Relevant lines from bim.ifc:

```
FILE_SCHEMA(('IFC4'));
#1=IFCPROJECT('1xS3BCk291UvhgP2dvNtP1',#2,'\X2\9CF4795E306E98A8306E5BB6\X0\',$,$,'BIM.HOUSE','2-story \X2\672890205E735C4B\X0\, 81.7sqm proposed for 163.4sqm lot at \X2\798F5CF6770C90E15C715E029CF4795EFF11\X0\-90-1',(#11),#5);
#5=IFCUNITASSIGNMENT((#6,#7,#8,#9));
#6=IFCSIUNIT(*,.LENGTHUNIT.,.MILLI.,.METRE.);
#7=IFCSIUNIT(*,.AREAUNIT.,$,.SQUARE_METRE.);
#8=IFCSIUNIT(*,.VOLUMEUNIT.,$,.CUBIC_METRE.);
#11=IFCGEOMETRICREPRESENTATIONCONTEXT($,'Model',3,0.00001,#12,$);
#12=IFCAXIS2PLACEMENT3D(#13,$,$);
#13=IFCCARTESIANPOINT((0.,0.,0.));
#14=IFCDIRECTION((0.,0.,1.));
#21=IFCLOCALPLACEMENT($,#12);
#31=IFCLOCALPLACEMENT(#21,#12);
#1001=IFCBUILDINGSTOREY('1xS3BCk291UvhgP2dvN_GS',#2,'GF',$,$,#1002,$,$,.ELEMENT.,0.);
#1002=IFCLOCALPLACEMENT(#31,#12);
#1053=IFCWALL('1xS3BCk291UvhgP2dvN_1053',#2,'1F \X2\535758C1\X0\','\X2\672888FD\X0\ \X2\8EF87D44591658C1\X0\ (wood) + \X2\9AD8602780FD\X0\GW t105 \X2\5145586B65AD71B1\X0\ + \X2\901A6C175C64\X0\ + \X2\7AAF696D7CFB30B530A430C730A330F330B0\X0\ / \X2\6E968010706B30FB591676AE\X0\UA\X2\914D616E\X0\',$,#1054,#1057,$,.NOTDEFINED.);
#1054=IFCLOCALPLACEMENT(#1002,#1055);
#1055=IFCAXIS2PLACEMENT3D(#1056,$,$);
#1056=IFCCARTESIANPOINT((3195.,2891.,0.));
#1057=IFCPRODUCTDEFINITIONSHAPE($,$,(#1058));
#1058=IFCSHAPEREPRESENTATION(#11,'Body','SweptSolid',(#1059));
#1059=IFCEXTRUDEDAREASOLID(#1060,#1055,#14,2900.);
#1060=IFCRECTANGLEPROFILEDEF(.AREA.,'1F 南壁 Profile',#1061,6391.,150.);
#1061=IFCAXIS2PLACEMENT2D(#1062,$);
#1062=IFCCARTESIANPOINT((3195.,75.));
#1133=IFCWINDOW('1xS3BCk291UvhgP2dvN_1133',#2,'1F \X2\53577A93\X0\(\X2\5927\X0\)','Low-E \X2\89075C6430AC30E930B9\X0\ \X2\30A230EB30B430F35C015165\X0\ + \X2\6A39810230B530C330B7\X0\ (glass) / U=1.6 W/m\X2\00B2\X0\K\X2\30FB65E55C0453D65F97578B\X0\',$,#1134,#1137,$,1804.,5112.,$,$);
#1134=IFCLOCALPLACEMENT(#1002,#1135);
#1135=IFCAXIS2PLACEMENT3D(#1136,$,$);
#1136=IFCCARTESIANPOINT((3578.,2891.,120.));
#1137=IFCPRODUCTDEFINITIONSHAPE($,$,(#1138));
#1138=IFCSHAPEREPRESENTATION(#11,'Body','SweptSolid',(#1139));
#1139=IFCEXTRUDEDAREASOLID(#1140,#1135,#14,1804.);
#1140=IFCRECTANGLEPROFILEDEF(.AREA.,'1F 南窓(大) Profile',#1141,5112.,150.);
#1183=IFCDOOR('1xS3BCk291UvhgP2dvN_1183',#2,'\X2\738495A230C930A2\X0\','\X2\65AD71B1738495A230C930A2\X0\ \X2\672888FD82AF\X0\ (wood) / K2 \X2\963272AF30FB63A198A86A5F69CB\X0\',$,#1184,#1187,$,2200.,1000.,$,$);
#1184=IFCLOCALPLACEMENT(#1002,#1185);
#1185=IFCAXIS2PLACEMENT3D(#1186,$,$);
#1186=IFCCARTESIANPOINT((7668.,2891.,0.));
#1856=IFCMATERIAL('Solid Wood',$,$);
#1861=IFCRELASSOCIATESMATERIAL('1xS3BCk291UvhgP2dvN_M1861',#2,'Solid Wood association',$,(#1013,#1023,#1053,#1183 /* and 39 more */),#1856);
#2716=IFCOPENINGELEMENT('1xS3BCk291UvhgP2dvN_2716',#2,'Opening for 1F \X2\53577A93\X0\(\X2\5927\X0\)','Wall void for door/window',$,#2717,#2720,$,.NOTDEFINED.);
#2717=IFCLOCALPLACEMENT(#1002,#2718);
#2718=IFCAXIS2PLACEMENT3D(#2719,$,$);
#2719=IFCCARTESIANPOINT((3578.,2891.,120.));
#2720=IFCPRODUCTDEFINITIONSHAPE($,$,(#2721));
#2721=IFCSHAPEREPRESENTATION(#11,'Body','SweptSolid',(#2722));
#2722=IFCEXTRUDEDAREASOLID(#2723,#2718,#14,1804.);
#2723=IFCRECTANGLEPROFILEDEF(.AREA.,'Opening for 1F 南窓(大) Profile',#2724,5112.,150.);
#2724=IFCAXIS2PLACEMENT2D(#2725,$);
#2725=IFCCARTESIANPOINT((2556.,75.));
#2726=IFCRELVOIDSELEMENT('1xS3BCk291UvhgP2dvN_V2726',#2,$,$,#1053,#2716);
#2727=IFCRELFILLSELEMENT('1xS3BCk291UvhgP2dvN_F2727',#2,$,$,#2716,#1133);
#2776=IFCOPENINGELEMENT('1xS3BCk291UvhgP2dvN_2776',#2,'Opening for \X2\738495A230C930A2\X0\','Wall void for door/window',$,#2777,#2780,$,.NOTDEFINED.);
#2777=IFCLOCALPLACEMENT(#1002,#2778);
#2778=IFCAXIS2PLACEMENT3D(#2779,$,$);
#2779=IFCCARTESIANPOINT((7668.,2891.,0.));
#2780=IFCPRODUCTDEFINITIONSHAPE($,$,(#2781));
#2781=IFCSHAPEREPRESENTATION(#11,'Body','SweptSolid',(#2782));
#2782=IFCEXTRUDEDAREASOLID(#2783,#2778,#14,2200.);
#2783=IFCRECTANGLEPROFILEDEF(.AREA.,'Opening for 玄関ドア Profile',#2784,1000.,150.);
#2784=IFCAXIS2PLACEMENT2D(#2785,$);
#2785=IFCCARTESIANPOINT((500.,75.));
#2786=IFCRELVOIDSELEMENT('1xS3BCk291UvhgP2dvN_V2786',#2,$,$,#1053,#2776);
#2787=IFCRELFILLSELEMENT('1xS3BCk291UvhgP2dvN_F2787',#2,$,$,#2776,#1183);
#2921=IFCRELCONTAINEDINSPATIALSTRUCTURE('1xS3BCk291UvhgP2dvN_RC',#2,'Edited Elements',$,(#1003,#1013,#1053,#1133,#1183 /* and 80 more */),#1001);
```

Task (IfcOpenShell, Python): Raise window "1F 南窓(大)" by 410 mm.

```python
import numpy as np
import ifcopenshell
import ifcopenshell.api.geometry
import ifcopenshell.util.placement
import ifcopenshell.util.unit

model = ifcopenshell.open("bim.ifc")
unit_scale = ifcopenshell.util.unit.calculate_unit_scale(model)

window = model.by_guid("1xS3BCk291UvhgP2dvN_1133")
opening = window.FillsVoids[0].RelatingOpeningElement
dz = 0.41 / unit_scale

shift = np.array([0.0, 0.0, dz])
# The window is not placed relative to its opening, so move both.
for product in (opening, window):
    matrix = ifcopenshell.util.placement.get_local_placement(product.ObjectPlacement)
    matrix[:3, 3] += shift
    ifcopenshell.api.geometry.edit_object_placement(model, product=product, matrix=matrix, is_si=False)

print(f"moved by {dz * unit_scale:+.3f} m")

model.write("bim_updated.ifc")
```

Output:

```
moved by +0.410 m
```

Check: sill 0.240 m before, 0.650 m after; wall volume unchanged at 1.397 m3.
